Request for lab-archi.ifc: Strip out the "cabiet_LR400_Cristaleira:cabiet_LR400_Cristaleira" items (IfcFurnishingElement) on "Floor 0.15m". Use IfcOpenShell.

First a look at what the model holds.

```python
import ifcopenshell
import ifcopenshell.util.element

model = ifcopenshell.open("lab-archi.ifc")
print(model.schema)
storey = next(s for s in model.by_type("IfcBuildingStorey") if s.Name == "Floor 0.15m")
furniture = [e for e in ifcopenshell.util.element.get_decomposition(storey) if e.is_a("IfcFurnishingElement")]
seen = {}
for e in furniture:
    element_type = ifcopenshell.util.element.get_type(e)
    name = element_type.Name if element_type not in (None, e) else None
    seen[name] = seen.get(name, 0) + 1
for name, count in sorted(seen.items(), key=str):
    print(count, "x", name)
```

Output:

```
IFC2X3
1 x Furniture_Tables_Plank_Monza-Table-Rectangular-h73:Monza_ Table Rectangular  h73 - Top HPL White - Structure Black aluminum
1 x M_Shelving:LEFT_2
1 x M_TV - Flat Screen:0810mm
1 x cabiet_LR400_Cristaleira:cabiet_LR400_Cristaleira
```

```python
import ifcopenshell
import ifcopenshell.api.root
import ifcopenshell.util.element

model = ifcopenshell.open("lab-archi.ifc")

storey = next(s for s in model.by_type("IfcBuildingStorey") if s.Name == "Floor 0.15m")
furniture = [e for e in ifcopenshell.util.element.get_decomposition(storey) if e.is_a("IfcFurnishingElement")]
targets = [e for e in furniture if (t := ifcopenshell.util.element.get_type(e)) not in (None, e) and t.Name == "cabiet_LR400_Cristaleira:cabiet_LR400_Cristaleira"]

for e in targets:
    ifcopenshell.api.root.remove_product(model, product=e)
print(len(targets), "removed")

model.write("lab-archi-out.ifc")
```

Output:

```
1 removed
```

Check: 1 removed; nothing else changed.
